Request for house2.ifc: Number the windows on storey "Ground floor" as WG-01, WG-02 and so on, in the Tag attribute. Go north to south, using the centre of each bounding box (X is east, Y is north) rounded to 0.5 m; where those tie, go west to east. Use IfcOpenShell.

First a look at what the model holds.

```python
import ifcopenshell
import ifcopenshell.util.element
import ifcopenshell.util.placement

model = ifcopenshell.open("house2.ifc")
print(model.schema)
storey = next(s for s in model.by_type("IfcBuildingStorey") if s.Name == "Ground floor")
windows = [e for e in ifcopenshell.util.element.get_decomposition(storey) if e.is_a("IfcWindow")]
for e in sorted(windows, key=lambda e: e.id()):
    origin = ifcopenshell.util.placement.get_local_placement(e.ObjectPlacement)[:3, 3]
    print(e.id(), e.Tag, e.Name, origin.round(2) + 0.0, sep=" | ")
```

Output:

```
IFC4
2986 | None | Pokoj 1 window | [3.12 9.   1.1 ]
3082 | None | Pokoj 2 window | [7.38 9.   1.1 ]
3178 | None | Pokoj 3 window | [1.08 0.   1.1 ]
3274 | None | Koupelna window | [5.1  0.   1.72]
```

```python
import ifcopenshell
import ifcopenshell.geom
import ifcopenshell.util.element
import ifcopenshell.util.shape

model = ifcopenshell.open("house2.ifc")
settings = ifcopenshell.geom.settings()
settings.set("use-world-coords", True)


def centre(element):
    shape = ifcopenshell.geom.create_shape(settings, element)
    return ifcopenshell.util.shape.get_bbox_centroid(shape.geometry)


storey = next(s for s in model.by_type("IfcBuildingStorey") if s.Name == "Ground floor")
windows = [e for e in ifcopenshell.util.element.get_decomposition(storey) if e.is_a("IfcWindow")]

# Insertion points can sit at a corner or the storey origin, so sort by the geometry (in metres).
centres = {e: centre(e) for e in windows}
windows.sort(key=lambda e: (-round(centres[e][1] / 0.5), centres[e][0]))

for i, e in enumerate(windows, start=1):
    number = f"WG-{i:02d}"
    e.Tag = number
    print(e.id(), number)

model.write("house2_v2.ifc")
```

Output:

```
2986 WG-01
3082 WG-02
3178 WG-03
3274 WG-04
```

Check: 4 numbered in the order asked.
